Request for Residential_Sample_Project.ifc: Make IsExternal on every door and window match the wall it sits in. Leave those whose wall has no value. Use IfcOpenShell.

First a look at what the model holds.

```python
import ifcopenshell
import ifcopenshell.util.element

model = ifcopenshell.open("Residential_Sample_Project.ifc")
print(model.schema)
seen = {}
for e in model.by_type("IfcDoor") + model.by_type("IfcWindow"):
    if not e.FillsVoids:
        continue
    host = e.FillsVoids[0].RelatingOpeningElement.VoidsElements[0].RelatingBuildingElement
    own = ifcopenshell.util.element.get_pset(e, f"Pset_{e.is_a()[3:].removesuffix('StandardCase')}Common", "IsExternal")
    wall = ifcopenshell.util.element.get_pset(host, "Pset_WallCommon", "IsExternal")
    seen[e.is_a(), own, wall] = seen.get((e.is_a(), own, wall), 0) + 1
for (cls, own, wall), count in sorted(seen.items(), key=str):
    print(count, cls, "IsExternal:", own, "| host wall:", wall)
```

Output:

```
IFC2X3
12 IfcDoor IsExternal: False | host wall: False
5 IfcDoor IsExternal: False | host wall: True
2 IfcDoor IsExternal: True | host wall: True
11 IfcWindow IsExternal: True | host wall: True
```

```python
import ifcopenshell
import ifcopenshell.api.pset
import ifcopenshell.util.element

model = ifcopenshell.open("Residential_Sample_Project.ifc")

count = 0
for ifc_class, pset_name in (("IfcDoor", "Pset_DoorCommon"), ("IfcWindow", "Pset_WindowCommon")):
    for e in model.by_type(ifc_class):
        if not e.FillsVoids:
            continue
        host = e.FillsVoids[0].RelatingOpeningElement.VoidsElements[0].RelatingBuildingElement
        external = ifcopenshell.util.element.get_pset(host, "Pset_WallCommon", "IsExternal")
        if external is None or ifcopenshell.util.element.get_pset(e, pset_name, "IsExternal") == external:
            continue
        pset = ifcopenshell.api.pset.add_pset(model, product=e, name=pset_name)
        ifcopenshell.api.pset.edit_pset(model, pset=pset, properties={"IsExternal": external})
        count += 1

print(count, "updated")

model.write("Residential_Sample_Project_rev.ifc")
```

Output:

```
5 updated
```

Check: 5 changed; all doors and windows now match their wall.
